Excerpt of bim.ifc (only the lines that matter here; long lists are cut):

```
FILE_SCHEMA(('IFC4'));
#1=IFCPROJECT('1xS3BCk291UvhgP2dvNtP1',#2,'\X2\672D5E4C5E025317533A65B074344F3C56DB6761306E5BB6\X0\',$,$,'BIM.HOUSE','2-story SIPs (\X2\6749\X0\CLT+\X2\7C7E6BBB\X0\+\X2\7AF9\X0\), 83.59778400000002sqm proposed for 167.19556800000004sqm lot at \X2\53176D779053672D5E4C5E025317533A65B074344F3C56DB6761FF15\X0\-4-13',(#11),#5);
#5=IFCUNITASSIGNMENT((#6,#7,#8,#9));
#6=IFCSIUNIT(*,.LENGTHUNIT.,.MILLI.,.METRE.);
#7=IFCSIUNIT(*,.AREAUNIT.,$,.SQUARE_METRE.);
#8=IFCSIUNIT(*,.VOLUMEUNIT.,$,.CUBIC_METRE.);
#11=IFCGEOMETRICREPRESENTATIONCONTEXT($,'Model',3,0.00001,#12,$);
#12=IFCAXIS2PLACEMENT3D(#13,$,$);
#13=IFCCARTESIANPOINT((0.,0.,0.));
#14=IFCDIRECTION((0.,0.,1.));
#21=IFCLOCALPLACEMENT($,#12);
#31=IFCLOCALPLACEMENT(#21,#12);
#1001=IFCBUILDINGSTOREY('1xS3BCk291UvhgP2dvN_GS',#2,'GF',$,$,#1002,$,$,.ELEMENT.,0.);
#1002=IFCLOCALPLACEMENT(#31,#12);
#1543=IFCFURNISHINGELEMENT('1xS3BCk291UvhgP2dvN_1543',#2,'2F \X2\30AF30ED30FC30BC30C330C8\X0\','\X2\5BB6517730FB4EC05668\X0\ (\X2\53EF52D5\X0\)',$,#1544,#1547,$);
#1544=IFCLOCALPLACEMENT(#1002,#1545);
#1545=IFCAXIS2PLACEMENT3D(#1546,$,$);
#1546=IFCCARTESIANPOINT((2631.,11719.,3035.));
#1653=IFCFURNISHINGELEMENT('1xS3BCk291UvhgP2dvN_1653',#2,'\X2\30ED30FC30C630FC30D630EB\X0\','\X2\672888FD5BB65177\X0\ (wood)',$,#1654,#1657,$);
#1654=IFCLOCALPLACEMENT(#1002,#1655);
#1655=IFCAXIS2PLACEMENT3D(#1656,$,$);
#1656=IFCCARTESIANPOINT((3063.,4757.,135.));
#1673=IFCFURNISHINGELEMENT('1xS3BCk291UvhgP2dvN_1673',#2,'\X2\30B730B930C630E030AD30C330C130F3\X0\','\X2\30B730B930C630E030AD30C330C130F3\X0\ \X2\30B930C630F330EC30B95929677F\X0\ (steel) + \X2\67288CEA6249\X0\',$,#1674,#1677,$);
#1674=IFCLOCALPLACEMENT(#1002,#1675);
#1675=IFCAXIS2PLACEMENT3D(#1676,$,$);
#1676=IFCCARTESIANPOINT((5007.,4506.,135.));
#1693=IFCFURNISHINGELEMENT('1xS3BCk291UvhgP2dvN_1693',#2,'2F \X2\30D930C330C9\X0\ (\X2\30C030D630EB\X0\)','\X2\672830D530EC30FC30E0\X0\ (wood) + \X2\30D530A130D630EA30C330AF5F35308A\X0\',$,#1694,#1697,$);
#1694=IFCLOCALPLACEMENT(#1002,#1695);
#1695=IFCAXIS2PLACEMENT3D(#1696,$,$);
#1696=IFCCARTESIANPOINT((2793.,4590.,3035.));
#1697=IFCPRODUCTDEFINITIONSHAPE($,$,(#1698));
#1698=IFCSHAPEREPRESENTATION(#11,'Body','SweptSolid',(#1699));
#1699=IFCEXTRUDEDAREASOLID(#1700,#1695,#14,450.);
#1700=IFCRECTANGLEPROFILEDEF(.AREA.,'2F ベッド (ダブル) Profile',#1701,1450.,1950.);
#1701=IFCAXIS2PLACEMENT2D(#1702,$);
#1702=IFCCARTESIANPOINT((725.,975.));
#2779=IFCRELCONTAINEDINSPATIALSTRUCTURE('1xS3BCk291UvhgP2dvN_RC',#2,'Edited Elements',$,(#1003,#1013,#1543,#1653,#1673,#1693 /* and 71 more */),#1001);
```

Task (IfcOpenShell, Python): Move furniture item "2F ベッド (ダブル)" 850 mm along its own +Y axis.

```python
import ifcopenshell
import ifcopenshell.api.geometry
import ifcopenshell.util.placement

model = ifcopenshell.open("bim.ifc")

item = model.by_guid("1xS3BCk291UvhgP2dvN_1693")
matrix = ifcopenshell.util.placement.get_local_placement(item.ObjectPlacement)
matrix[:3, 3] += matrix[:3, 1] * 850.0
ifcopenshell.api.geometry.edit_object_placement(model, product=item, matrix=matrix, is_si=False)

print(ifcopenshell.util.placement.get_local_placement(item.ObjectPlacement).round(3) + 0.0)

model.write("bim_edited.ifc")
```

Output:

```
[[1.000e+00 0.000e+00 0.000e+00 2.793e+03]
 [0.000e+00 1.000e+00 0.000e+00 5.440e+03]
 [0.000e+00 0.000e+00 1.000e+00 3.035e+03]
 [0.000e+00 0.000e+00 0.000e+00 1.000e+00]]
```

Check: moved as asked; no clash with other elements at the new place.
